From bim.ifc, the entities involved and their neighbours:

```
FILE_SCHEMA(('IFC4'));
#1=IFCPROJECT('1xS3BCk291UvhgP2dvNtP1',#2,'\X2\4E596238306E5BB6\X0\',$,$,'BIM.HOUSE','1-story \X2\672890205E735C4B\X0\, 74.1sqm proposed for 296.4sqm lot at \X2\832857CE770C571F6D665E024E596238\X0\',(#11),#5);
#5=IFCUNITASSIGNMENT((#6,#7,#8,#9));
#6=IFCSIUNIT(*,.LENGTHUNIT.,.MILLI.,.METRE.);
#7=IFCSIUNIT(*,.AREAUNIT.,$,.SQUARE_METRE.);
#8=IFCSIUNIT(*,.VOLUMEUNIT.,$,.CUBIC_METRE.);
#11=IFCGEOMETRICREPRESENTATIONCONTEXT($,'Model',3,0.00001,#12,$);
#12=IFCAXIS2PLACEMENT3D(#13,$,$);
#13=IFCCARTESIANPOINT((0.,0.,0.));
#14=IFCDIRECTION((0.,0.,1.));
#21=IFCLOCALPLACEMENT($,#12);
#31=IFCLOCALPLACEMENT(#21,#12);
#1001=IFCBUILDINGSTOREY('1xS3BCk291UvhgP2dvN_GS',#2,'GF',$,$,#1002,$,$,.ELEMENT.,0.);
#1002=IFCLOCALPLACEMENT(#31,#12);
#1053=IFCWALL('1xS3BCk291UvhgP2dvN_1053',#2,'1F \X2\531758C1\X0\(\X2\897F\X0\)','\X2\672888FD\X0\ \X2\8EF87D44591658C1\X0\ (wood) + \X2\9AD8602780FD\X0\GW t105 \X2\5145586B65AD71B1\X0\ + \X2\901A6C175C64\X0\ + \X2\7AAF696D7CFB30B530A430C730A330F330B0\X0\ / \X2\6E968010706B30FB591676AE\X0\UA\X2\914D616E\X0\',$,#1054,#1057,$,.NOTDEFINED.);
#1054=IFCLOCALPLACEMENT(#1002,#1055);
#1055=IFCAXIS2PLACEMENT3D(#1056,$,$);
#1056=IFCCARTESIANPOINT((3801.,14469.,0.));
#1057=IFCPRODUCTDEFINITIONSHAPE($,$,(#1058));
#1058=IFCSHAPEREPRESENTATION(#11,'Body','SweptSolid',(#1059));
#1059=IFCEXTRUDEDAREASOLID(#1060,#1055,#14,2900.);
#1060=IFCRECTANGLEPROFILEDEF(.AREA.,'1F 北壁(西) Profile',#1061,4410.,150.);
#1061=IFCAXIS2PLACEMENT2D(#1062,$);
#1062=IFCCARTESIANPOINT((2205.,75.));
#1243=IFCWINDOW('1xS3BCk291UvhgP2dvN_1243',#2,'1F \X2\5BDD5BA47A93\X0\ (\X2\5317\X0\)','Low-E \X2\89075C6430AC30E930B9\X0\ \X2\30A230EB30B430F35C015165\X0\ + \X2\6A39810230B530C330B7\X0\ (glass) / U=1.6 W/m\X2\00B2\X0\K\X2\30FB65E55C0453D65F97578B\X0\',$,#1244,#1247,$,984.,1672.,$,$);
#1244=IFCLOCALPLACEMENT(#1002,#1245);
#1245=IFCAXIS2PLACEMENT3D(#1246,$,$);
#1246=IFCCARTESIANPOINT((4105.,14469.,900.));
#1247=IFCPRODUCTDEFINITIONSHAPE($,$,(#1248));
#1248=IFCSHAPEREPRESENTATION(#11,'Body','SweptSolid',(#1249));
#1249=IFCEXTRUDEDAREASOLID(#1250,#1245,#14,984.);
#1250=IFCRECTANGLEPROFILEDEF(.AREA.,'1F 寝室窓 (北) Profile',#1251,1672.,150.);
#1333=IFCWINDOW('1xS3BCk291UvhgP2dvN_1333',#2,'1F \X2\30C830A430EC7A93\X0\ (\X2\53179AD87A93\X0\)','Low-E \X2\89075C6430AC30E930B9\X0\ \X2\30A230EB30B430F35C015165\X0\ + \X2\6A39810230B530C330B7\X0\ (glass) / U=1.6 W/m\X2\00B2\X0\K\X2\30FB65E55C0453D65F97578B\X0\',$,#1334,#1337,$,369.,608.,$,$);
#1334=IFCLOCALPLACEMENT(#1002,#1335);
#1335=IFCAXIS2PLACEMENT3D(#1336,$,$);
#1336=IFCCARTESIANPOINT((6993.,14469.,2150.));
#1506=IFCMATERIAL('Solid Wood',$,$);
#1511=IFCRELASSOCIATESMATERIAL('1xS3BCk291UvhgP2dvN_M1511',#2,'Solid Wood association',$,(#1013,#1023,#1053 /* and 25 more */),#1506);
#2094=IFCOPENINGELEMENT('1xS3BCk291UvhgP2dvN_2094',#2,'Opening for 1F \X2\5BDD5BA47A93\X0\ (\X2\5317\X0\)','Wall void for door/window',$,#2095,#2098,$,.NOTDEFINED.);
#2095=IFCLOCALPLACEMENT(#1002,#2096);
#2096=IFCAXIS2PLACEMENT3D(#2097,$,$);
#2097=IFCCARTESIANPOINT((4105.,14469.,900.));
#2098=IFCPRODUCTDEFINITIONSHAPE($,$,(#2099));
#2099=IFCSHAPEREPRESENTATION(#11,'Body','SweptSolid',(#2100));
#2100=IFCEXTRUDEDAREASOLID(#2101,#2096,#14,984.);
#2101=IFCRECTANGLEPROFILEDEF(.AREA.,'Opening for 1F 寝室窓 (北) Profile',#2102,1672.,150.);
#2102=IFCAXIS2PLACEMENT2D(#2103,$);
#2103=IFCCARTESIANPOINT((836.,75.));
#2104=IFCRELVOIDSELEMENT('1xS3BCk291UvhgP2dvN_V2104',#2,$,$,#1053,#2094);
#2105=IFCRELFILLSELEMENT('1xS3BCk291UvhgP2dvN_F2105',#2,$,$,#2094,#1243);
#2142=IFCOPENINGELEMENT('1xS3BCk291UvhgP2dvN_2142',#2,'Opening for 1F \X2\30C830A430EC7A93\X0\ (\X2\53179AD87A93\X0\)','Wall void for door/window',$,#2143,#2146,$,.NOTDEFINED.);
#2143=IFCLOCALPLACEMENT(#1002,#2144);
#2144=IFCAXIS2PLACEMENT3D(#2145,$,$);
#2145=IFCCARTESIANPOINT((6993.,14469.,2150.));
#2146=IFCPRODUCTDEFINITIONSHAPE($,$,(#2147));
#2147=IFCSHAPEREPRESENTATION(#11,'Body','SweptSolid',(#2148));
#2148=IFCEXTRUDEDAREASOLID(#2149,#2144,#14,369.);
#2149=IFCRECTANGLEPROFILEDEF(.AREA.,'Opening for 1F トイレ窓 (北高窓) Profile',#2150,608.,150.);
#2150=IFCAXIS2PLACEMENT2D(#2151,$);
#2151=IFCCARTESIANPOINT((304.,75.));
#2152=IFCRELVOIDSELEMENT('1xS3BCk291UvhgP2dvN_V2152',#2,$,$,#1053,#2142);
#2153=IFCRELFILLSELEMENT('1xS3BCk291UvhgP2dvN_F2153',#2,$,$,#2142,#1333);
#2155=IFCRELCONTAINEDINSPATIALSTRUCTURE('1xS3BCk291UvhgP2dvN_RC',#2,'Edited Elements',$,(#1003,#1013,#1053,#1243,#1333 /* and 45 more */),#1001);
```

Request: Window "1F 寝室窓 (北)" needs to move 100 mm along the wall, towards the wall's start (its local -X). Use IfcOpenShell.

```python
import ifcopenshell
import ifcopenshell.api.geometry
import ifcopenshell.util.placement

model = ifcopenshell.open("bim.ifc")

window = model.by_guid("1xS3BCk291UvhgP2dvN_1243")
opening = window.FillsVoids[0].RelatingOpeningElement
wall = opening.VoidsElements[0].RelatingBuildingElement

wall_matrix = ifcopenshell.util.placement.get_local_placement(wall.ObjectPlacement)
shift = wall_matrix[:3, 0] * -100.0
before = ifcopenshell.util.placement.get_local_placement(window.ObjectPlacement)[:3, 3].copy()

# The window is not placed relative to its opening, so move both.
for product in (opening, window):
    matrix = ifcopenshell.util.placement.get_local_placement(product.ObjectPlacement)
    matrix[:3, 3] += shift
    ifcopenshell.api.geometry.edit_object_placement(model, product=product, matrix=matrix, is_si=False)

after = ifcopenshell.util.placement.get_local_placement(window.ObjectPlacement)[:3, 3]
print("window moved by", (after - before).round(3) + 0.0)

model.write("bim_updated.ifc")
```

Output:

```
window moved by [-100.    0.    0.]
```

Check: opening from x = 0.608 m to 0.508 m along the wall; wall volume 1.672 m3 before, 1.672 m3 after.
